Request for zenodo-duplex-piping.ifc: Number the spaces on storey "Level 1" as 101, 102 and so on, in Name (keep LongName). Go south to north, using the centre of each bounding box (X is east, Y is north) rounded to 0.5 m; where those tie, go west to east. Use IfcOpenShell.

First a look at what the model holds.

```python
import ifcopenshell
import ifcopenshell.util.element
import ifcopenshell.util.placement

model = ifcopenshell.open("zenodo-duplex-piping.ifc")
print(model.schema)
storey = next(s for s in model.by_type("IfcBuildingStorey") if s.Name == "Level 1")
spaces = [e for e in ifcopenshell.util.element.get_decomposition(storey) if e.is_a("IfcSpace")]
for e in sorted(spaces, key=lambda e: e.id()):
    origin = ifcopenshell.util.placement.get_local_placement(e.ObjectPlacement)[:3, 3]
    print(e.id(), e.Name, e.LongName, origin.round(2) + 0.0, sep=" | ")
```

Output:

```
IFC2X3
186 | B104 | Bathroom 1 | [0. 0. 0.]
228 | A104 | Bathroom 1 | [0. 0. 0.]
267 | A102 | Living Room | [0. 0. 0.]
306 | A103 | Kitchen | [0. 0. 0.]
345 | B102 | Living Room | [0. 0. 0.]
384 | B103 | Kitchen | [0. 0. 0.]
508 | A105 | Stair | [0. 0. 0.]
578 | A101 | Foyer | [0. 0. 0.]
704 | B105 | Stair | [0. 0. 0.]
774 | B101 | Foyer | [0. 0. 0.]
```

```python
import ifcopenshell
import ifcopenshell.geom
import ifcopenshell.util.element
import ifcopenshell.util.shape

model = ifcopenshell.open("zenodo-duplex-piping.ifc")
settings = ifcopenshell.geom.settings()
settings.set("use-world-coords", True)


def centre(element):
    shape = ifcopenshell.geom.create_shape(settings, element)
    return ifcopenshell.util.shape.get_bbox_centroid(shape.geometry)


storey = next(s for s in model.by_type("IfcBuildingStorey") if s.Name == "Level 1")
spaces = [e for e in ifcopenshell.util.element.get_decomposition(storey) if e.is_a("IfcSpace")]

# Insertion points can sit at a corner or the storey origin, so sort by the geometry (in metres).
centres = {e: centre(e) for e in spaces}
spaces.sort(key=lambda e: (round(centres[e][1] / 0.5), centres[e][0]))

for i, e in enumerate(spaces, start=1):
    number = f"1{i:02d}"
    e.Name = number
    print(e.id(), number)

model.write("zenodo-duplex-piping_edited.ifc")
```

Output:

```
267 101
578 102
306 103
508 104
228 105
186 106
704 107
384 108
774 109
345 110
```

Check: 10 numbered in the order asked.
